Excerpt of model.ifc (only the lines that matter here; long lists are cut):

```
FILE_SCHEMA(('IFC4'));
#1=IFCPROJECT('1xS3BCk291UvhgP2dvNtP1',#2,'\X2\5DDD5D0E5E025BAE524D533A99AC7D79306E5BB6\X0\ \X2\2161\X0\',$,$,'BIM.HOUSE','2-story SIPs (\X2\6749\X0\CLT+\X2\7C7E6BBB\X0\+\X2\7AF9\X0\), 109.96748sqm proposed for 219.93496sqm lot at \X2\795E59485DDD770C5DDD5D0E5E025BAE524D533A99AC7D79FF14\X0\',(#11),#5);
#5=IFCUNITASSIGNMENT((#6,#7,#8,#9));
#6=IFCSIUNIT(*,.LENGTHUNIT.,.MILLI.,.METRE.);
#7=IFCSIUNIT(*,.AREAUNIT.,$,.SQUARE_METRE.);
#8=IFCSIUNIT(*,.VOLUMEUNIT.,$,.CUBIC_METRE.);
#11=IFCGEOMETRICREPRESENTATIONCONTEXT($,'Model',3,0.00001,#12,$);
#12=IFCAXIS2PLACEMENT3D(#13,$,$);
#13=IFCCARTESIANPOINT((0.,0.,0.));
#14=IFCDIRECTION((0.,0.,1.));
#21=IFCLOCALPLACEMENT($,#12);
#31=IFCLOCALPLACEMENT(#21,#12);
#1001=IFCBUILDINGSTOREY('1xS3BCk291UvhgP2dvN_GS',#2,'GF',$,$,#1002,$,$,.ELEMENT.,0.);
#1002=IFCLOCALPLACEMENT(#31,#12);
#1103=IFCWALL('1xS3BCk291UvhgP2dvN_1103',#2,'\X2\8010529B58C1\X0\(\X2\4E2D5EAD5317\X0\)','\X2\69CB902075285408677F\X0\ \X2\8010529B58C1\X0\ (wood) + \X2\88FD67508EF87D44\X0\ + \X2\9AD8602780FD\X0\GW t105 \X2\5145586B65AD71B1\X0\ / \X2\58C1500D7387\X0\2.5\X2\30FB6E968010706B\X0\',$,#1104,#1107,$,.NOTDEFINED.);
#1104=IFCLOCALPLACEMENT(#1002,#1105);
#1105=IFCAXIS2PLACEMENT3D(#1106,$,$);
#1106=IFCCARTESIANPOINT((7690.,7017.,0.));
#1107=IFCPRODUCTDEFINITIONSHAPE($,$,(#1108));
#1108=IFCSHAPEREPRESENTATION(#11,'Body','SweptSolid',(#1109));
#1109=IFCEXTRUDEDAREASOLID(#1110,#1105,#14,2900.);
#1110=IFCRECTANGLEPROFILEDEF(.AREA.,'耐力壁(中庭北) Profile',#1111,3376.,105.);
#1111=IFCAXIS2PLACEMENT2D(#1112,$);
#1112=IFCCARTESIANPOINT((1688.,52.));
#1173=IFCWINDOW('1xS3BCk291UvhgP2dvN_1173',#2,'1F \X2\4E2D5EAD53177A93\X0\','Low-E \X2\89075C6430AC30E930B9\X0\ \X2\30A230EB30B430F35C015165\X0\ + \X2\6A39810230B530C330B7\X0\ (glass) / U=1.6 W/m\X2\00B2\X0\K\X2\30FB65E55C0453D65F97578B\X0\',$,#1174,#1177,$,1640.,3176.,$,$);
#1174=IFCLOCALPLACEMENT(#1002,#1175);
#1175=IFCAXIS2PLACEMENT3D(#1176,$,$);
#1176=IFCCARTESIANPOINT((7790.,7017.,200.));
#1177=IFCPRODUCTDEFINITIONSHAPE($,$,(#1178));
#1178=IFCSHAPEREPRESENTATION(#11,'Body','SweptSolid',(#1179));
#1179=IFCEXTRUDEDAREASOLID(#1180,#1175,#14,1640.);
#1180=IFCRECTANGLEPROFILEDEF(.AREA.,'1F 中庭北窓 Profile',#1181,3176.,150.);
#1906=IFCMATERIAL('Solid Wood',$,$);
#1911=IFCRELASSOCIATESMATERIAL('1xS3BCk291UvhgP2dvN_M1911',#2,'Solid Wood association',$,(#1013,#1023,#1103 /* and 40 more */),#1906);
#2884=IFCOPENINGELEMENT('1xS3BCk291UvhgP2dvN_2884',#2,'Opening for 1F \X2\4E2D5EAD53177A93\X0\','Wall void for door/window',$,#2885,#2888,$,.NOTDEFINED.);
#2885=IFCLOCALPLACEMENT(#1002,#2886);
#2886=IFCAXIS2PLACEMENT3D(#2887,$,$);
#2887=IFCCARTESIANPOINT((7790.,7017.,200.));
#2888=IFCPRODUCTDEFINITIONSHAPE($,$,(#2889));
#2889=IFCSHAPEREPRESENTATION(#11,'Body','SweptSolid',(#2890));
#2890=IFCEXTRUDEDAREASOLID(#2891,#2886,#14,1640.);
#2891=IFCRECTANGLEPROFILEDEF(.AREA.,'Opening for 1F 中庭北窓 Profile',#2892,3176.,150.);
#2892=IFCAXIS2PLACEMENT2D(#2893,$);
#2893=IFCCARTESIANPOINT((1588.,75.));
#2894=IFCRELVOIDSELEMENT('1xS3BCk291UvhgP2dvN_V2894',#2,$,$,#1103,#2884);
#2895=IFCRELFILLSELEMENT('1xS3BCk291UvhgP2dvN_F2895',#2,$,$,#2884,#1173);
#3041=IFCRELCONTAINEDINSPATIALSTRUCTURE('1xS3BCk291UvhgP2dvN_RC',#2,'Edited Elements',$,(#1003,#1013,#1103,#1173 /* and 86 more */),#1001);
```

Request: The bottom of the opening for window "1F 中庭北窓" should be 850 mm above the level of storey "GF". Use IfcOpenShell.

```python
import numpy as np
import ifcopenshell
import ifcopenshell.api.geometry
import ifcopenshell.geom
import ifcopenshell.util.element
import ifcopenshell.util.placement
import ifcopenshell.util.shape
import ifcopenshell.util.unit

model = ifcopenshell.open("model.ifc")
unit_scale = ifcopenshell.util.unit.calculate_unit_scale(model)

window = model.by_id(1173)
opening = window.FillsVoids[0].RelatingOpeningElement
storey = ifcopenshell.util.element.get_container(window, ifc_class="IfcBuildingStorey")
level = ifcopenshell.util.placement.get_local_placement(storey.ObjectPlacement)[2, 3]

# The opening's origin need not be at the sill, so measure its lowest point.
shape = ifcopenshell.geom.create_shape(ifcopenshell.geom.settings(), opening)
bottom = ifcopenshell.util.shape.get_shape_bottom_elevation(shape, shape.geometry) / unit_scale
dz = level + 0.85 / unit_scale - bottom

shift = np.array([0.0, 0.0, dz])
# The window is not placed relative to its opening, so move both.
for product in (opening, window):
    matrix = ifcopenshell.util.placement.get_local_placement(product.ObjectPlacement)
    matrix[:3, 3] += shift
    ifcopenshell.api.geometry.edit_object_placement(model, product=product, matrix=matrix, is_si=False)

print(f"moved by {dz * unit_scale:+.3f} m")

model.write("model_rev.ifc")
```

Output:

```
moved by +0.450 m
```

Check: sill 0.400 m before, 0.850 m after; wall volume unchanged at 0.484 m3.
